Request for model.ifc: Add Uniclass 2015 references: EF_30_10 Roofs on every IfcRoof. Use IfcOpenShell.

First a look at what the model holds.

```python
import ifcopenshell

model = ifcopenshell.open("model.ifc")
print(model.schema)
print("classifications:", [c.Name for c in model.by_type("IfcClassification")])
for ifc_class in ("IfcDoor", "IfcRoof", "IfcStair", "IfcWall", "IfcWindow"):
    print(ifc_class, len(model.by_type(ifc_class)))
```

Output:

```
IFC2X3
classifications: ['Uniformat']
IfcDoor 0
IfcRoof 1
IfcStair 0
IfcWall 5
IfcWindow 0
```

```python
import ifcopenshell
import ifcopenshell.api.classification

model = ifcopenshell.open("model.ifc")

# IFC2X3 requires Source and Edition and has no link from the project to the system.
system = model.create_entity("IfcClassification", Source="NBS", Edition="2015", Name="Uniclass 2015")

codes = {
    "IfcRoof": ("EF_30_10", "Roofs"),
}
for ifc_class, (code, name) in codes.items():
    products = model.by_type(ifc_class)
    ifcopenshell.api.classification.add_reference(
        model, products=products, classification=system, identification=code, name=name
    )
    print(code, len(products))

model.write("model_rev.ifc")
```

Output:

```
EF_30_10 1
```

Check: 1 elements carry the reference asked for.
